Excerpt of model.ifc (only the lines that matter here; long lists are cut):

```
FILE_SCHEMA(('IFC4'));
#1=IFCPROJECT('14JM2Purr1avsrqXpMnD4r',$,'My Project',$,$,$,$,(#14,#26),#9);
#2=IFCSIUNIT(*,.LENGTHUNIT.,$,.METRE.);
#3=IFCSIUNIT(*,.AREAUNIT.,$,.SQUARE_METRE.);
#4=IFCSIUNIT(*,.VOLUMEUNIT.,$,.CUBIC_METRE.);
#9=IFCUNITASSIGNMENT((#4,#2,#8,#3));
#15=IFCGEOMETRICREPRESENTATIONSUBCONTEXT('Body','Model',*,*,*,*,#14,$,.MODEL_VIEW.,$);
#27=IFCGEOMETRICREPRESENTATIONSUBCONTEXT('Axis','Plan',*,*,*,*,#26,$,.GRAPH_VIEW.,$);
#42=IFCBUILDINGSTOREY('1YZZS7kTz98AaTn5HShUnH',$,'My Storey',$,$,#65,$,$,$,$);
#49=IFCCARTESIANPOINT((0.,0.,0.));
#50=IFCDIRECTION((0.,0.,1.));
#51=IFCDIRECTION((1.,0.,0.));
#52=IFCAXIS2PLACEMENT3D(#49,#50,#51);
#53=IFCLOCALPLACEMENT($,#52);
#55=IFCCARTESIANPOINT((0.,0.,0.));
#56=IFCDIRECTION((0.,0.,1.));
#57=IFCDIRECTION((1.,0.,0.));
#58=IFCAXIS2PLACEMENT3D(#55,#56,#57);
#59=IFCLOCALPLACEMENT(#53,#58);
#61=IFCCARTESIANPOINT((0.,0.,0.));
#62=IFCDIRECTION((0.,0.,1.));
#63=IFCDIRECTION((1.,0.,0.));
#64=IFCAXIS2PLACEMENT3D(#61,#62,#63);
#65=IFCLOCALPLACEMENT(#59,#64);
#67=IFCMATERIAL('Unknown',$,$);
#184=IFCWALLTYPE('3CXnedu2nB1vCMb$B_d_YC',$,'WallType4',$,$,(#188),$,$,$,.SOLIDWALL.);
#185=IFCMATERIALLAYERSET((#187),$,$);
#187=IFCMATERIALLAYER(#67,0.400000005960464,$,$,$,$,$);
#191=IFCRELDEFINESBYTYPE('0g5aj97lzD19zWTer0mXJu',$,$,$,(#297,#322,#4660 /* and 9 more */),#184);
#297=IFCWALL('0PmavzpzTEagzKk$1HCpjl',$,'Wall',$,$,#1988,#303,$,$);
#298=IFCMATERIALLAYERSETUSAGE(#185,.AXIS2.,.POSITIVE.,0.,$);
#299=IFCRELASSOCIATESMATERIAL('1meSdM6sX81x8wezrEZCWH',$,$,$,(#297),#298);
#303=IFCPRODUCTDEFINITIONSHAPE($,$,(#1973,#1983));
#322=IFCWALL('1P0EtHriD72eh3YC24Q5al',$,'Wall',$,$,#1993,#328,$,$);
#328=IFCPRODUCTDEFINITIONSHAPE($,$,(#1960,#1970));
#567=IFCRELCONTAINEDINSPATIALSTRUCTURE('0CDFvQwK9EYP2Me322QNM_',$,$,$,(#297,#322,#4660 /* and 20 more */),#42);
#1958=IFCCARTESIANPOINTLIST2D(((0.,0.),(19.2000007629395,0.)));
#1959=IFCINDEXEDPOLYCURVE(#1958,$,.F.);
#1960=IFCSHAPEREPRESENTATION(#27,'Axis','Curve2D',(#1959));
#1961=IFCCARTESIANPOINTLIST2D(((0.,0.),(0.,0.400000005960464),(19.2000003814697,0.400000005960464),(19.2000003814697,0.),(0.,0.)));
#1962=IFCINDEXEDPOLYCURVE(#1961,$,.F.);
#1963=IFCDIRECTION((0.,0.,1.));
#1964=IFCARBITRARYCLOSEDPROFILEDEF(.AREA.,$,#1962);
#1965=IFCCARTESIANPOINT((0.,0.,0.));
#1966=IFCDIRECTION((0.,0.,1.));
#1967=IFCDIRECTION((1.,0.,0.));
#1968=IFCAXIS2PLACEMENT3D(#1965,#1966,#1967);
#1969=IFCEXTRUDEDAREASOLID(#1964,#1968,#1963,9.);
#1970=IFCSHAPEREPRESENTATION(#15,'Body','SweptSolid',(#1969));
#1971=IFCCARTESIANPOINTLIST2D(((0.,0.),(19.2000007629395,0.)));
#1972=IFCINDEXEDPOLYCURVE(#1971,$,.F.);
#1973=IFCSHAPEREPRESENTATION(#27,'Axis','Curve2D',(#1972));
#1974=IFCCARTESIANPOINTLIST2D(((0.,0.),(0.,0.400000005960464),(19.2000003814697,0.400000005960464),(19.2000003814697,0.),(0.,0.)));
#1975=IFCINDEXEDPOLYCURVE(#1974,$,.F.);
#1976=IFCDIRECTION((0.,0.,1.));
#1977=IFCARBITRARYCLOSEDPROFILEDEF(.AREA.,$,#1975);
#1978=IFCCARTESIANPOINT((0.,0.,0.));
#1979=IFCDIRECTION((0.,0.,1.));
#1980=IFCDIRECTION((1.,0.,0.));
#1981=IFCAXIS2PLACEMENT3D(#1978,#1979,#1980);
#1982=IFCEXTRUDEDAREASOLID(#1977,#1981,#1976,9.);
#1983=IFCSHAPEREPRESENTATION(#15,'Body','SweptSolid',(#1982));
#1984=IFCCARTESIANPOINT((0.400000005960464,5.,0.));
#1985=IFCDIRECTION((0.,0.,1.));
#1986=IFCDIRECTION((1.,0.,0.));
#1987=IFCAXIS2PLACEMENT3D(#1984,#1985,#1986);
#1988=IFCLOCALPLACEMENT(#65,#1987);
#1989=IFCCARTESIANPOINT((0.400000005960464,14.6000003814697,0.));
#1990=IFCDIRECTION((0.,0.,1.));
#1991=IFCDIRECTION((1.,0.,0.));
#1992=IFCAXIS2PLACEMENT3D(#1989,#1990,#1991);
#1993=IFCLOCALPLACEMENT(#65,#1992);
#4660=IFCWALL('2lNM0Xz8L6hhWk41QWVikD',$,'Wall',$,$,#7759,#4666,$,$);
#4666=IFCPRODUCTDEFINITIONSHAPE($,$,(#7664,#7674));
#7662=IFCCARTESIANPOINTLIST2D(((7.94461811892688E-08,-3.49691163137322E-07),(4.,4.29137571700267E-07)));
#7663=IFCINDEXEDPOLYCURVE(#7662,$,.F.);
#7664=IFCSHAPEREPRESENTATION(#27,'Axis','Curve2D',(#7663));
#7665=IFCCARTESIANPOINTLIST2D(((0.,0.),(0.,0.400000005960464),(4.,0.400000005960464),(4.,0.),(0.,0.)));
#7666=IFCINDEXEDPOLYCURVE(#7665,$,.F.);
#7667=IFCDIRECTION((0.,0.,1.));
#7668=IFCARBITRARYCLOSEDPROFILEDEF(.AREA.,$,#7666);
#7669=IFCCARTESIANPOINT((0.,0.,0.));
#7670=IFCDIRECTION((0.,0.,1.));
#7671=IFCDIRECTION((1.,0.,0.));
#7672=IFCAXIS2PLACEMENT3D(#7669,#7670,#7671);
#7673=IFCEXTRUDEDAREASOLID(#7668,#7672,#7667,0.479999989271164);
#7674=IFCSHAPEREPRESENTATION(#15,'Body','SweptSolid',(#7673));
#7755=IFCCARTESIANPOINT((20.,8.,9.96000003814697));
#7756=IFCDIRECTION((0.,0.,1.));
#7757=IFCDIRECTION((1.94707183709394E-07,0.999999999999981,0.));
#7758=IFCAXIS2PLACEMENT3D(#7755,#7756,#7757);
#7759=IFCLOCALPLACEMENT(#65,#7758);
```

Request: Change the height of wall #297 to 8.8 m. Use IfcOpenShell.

```python
import ifcopenshell
import ifcopenshell.geom
import ifcopenshell.util.representation
import ifcopenshell.util.shape
import ifcopenshell.util.unit

model = ifcopenshell.open("model.ifc")
unit_scale = ifcopenshell.util.unit.calculate_unit_scale(model)
settings = ifcopenshell.geom.settings()


def volume(element):
    """Net volume in cubic metres, openings subtracted."""
    shape = ifcopenshell.geom.create_shape(settings, element)
    return ifcopenshell.util.shape.get_volume(shape.geometry)


wall = model.by_guid("0PmavzpzTEagzKk$1HCpjl")
before = volume(wall)

body = ifcopenshell.util.representation.get_representation(wall, "Model", "Body")
solid = body.Items[0]
old_height = solid.Depth
solid.Depth = 8.8 / unit_scale
after = volume(wall)

print(f"height {old_height:g} -> {solid.Depth:g}, volume {before:.3f} -> {after:.3f} m3")

model.write("model_edited.ifc")
```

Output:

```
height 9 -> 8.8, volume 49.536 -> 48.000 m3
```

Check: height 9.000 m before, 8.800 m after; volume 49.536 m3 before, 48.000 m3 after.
